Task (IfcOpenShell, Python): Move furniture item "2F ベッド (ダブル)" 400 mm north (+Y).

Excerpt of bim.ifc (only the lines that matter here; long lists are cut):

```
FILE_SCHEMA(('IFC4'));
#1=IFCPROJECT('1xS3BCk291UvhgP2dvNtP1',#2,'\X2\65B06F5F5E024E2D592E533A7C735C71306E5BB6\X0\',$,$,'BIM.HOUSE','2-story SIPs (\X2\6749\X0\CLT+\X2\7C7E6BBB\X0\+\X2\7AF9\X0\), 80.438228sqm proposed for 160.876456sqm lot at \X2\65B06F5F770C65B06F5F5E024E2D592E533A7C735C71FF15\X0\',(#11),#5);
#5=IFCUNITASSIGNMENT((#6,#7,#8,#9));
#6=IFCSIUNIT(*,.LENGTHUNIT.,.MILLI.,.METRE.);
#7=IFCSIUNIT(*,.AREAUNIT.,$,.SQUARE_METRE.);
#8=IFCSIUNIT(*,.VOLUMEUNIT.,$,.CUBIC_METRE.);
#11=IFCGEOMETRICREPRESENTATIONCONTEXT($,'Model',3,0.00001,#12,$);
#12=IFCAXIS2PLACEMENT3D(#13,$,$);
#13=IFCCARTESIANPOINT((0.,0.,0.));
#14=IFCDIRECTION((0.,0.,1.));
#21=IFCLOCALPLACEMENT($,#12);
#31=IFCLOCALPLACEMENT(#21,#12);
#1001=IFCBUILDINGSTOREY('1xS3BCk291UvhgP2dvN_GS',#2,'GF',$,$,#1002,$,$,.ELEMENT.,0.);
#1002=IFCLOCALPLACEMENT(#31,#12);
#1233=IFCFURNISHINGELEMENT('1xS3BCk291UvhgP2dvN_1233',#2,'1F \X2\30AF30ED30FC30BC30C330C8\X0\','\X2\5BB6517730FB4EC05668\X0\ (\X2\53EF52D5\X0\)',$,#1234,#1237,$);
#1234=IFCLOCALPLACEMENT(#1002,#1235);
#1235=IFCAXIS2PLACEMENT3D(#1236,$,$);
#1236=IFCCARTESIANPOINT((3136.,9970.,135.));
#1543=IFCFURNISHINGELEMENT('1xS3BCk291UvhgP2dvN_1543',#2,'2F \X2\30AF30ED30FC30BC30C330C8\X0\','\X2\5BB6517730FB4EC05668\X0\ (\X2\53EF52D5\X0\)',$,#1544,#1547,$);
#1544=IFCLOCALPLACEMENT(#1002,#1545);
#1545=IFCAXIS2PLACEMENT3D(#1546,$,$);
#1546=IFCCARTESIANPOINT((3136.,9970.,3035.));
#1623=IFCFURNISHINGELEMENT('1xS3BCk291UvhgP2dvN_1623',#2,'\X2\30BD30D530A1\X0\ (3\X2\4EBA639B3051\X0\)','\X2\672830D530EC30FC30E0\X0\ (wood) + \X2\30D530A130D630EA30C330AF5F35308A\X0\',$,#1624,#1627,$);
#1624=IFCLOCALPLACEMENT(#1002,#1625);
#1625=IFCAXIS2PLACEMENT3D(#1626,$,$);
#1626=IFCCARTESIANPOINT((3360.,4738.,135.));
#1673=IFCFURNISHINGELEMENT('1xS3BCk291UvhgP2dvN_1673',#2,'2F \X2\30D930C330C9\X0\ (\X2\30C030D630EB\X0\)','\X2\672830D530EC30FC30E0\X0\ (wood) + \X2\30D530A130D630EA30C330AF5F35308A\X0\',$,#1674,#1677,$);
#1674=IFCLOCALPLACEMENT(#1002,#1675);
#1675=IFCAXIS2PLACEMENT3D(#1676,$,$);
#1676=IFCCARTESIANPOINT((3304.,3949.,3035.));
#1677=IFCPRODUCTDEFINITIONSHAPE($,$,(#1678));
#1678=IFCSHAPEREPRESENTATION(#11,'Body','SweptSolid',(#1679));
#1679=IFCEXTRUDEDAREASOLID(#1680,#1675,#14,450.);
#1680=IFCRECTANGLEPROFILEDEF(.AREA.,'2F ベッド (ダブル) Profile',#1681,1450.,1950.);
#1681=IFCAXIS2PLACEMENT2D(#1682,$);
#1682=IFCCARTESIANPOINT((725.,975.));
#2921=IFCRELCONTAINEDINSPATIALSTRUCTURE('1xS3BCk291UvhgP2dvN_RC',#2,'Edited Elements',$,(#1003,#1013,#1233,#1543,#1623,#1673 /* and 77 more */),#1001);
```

```python
import ifcopenshell
import ifcopenshell.api.geometry
import ifcopenshell.util.placement

model = ifcopenshell.open("bim.ifc")

item = model.by_id(1673)
matrix = ifcopenshell.util.placement.get_local_placement(item.ObjectPlacement)
matrix[1, 3] += 400.0
ifcopenshell.api.geometry.edit_object_placement(model, product=item, matrix=matrix, is_si=False)

print(ifcopenshell.util.placement.get_local_placement(item.ObjectPlacement).round(3) + 0.0)

model.write("bim_edited.ifc")
```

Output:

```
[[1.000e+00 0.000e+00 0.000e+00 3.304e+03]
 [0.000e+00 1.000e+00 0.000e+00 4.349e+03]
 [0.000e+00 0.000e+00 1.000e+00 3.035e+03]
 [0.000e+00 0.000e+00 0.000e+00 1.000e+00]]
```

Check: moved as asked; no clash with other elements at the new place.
